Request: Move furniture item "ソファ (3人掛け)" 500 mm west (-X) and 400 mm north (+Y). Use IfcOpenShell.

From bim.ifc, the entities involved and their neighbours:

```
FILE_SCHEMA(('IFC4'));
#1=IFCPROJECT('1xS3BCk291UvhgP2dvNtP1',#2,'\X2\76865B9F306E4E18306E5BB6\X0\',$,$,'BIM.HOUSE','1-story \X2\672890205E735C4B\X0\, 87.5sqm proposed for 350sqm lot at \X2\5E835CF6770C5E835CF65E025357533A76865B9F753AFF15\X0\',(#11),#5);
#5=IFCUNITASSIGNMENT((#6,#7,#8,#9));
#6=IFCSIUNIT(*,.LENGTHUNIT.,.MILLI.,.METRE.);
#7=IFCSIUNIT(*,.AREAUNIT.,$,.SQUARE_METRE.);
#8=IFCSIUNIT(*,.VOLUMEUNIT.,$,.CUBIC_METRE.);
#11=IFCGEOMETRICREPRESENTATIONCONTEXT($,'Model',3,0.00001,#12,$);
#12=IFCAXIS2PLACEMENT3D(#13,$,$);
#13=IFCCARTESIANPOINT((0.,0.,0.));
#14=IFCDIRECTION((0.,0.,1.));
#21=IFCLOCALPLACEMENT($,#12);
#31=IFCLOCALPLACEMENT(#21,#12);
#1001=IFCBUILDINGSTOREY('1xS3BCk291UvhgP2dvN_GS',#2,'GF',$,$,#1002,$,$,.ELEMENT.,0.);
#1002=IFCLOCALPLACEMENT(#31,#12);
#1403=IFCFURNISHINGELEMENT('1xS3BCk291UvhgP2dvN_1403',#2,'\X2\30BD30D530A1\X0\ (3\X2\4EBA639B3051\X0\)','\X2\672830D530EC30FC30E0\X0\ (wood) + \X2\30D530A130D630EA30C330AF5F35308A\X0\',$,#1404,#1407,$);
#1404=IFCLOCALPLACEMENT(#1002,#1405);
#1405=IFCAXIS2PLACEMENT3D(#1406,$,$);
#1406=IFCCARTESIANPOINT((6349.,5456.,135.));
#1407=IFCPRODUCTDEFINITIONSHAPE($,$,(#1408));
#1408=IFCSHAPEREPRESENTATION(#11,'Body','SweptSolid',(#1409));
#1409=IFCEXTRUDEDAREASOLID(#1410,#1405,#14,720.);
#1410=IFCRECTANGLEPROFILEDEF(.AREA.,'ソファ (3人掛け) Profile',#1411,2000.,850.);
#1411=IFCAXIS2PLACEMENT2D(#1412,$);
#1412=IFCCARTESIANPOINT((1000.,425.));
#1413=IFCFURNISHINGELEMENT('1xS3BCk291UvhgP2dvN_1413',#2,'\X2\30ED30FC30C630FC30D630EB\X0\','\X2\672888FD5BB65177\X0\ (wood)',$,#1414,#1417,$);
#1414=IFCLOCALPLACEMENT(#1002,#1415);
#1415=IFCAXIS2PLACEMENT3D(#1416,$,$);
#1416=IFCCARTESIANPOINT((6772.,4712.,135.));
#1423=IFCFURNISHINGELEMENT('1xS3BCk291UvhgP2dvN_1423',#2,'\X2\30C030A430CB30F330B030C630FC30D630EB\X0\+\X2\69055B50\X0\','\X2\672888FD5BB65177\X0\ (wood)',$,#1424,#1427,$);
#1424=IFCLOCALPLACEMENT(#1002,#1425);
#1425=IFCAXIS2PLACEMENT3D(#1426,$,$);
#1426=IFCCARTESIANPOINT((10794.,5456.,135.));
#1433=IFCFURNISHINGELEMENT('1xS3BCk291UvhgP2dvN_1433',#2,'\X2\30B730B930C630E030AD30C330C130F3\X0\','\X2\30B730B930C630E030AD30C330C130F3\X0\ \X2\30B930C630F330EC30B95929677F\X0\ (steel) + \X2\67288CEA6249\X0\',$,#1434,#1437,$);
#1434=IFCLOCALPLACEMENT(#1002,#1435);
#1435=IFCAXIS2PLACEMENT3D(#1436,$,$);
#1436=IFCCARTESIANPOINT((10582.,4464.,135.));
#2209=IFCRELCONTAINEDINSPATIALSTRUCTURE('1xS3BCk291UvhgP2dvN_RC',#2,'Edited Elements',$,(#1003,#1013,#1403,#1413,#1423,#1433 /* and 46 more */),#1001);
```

```python
import ifcopenshell
import ifcopenshell.api.geometry
import ifcopenshell.util.placement

model = ifcopenshell.open("bim.ifc")

item = model.by_guid("1xS3BCk291UvhgP2dvN_1403")
matrix = ifcopenshell.util.placement.get_local_placement(item.ObjectPlacement)
matrix[0, 3] -= 500.0
matrix[1, 3] += 400.0
ifcopenshell.api.geometry.edit_object_placement(model, product=item, matrix=matrix, is_si=False)

print(ifcopenshell.util.placement.get_local_placement(item.ObjectPlacement).round(3) + 0.0)

model.write("bim_edited.ifc")
```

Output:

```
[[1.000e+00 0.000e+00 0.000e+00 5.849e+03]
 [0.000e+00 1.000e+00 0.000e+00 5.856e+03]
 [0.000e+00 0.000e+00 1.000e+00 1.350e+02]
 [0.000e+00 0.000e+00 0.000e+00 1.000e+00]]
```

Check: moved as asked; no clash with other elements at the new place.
